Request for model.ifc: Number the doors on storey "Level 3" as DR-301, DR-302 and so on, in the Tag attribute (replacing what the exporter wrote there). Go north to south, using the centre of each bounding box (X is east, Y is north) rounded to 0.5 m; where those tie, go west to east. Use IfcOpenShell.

First a look at what the model holds.

```python
import ifcopenshell
import ifcopenshell.util.element
import ifcopenshell.util.placement

model = ifcopenshell.open("model.ifc")
print(model.schema)
storey = next(s for s in model.by_type("IfcBuildingStorey") if s.Name == "Level 3")
doors = [e for e in ifcopenshell.util.element.get_decomposition(storey) if e.is_a("IfcDoor")]
for e in sorted(doors, key=lambda e: e.id()):
    origin = ifcopenshell.util.placement.get_local_placement(e.ObjectPlacement)[:3, 3]
    print(e.id(), e.Tag, e.Name, origin.round(2) + 0.0, sep=" | ")
```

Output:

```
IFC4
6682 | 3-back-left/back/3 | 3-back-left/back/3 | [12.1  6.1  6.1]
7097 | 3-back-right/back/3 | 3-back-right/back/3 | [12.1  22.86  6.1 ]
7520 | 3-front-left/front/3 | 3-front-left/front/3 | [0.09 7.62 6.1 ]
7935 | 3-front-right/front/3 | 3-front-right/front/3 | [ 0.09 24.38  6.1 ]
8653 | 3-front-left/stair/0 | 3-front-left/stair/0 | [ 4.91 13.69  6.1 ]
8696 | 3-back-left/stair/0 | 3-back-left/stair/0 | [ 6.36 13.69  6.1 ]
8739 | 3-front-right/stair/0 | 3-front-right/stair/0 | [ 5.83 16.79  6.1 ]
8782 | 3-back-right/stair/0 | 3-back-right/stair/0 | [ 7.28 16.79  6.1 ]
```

```python
import ifcopenshell
import ifcopenshell.geom
import ifcopenshell.util.element
import ifcopenshell.util.shape

model = ifcopenshell.open("model.ifc")
settings = ifcopenshell.geom.settings()
settings.set("use-world-coords", True)


def centre(element):
    shape = ifcopenshell.geom.create_shape(settings, element)
    return ifcopenshell.util.shape.get_bbox_centroid(shape.geometry)


storey = next(s for s in model.by_type("IfcBuildingStorey") if s.Name == "Level 3")
doors = [e for e in ifcopenshell.util.element.get_decomposition(storey) if e.is_a("IfcDoor")]

# Insertion points can sit at a corner or the storey origin, so sort by the geometry (in metres).
centres = {e: centre(e) for e in doors}
doors.sort(key=lambda e: (-round(centres[e][1] / 0.5), centres[e][0]))

for i, e in enumerate(doors, start=1):
    number = f"DR-3{i:02d}"
    e.Tag = number
    print(e.id(), number)

model.write("model_edited.ifc")
```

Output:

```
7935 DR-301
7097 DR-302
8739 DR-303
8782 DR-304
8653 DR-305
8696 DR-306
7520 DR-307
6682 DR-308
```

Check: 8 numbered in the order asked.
